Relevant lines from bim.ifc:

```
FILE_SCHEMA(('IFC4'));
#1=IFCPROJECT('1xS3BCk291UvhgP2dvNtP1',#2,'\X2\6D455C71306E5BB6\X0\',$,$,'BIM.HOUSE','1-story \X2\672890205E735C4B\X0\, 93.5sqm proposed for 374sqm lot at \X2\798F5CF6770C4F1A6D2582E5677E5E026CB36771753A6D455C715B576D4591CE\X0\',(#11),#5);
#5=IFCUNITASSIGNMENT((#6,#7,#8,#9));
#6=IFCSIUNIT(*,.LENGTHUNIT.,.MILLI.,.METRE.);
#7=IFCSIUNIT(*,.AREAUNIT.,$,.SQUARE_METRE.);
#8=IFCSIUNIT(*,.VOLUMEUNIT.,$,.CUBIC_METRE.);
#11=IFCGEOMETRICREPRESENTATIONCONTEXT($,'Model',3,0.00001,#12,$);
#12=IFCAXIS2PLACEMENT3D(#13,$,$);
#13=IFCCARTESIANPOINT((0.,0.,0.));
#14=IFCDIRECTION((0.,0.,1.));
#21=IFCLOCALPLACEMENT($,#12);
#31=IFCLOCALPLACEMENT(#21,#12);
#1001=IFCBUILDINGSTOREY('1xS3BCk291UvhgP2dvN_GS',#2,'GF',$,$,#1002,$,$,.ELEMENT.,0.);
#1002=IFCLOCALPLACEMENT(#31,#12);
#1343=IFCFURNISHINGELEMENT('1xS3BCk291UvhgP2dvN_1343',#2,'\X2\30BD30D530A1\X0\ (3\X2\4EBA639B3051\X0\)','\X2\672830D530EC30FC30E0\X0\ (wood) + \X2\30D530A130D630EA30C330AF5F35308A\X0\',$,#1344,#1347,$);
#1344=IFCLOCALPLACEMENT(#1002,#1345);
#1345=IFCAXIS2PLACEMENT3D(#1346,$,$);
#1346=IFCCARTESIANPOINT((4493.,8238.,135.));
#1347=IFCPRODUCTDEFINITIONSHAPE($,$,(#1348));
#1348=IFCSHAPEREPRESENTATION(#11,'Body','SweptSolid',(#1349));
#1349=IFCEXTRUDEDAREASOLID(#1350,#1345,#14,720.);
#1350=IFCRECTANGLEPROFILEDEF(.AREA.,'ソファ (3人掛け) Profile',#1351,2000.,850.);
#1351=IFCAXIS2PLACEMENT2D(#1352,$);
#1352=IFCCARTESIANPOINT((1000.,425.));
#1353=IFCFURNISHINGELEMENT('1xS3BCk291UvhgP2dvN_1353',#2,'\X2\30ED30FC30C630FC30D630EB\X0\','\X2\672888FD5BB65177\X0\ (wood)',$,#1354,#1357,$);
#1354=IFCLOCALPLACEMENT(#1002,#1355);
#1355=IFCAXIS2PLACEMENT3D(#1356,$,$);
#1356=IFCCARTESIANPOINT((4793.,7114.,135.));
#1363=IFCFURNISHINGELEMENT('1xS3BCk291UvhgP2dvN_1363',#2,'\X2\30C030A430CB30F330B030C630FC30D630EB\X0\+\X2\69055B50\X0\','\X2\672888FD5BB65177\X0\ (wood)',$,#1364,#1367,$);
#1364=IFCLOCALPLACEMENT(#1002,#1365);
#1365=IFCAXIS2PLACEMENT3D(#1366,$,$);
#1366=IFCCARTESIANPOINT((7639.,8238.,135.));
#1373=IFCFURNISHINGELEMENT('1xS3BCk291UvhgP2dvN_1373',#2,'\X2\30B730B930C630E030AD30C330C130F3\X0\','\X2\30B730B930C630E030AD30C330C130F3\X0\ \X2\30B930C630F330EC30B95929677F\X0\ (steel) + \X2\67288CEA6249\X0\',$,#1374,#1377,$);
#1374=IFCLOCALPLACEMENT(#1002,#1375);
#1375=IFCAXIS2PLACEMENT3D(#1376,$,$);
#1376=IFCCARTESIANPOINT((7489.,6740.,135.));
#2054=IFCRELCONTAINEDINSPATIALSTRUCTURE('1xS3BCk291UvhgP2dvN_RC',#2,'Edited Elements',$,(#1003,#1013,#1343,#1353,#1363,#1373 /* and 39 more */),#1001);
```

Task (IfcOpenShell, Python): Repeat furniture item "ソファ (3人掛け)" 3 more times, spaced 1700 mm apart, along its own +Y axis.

```python
import ifcopenshell
import ifcopenshell.api.geometry
import ifcopenshell.api.root
import ifcopenshell.util.element
import ifcopenshell.util.placement

model = ifcopenshell.open("bim.ifc")


def reuse_history(source, copy):
    """copy_class also copies each property set's owner history, people and application; keep the originals."""
    for rel in copy.IsDefinedBy:
        if rel.is_a("IfcRelDefinesByProperties") and (history := rel.RelatingPropertyDefinition.OwnerHistory):
            rel.RelatingPropertyDefinition.OwnerHistory = source.OwnerHistory
            ifcopenshell.util.element.remove_deep2(model, history)


source = model.by_guid("1xS3BCk291UvhgP2dvN_1343")
base = ifcopenshell.util.placement.get_local_placement(source.ObjectPlacement)
step = base[:3, 1] * 1700.0

for i in range(1, 4):
    copy = ifcopenshell.api.root.copy_class(model, product=source)
    copy.Representation = ifcopenshell.util.element.copy_deep(
        model, source.Representation, exclude=["IfcGeometricRepresentationContext", "IfcRepresentationMap"]
    )
    reuse_history(source, copy)
    matrix = base.copy()
    matrix[:3, 3] += i * step
    print("added at", matrix[:3, 3].round(3) + 0.0)
    ifcopenshell.api.geometry.edit_object_placement(model, product=copy, matrix=matrix, is_si=False)

model.write("bim_v2.ifc")
```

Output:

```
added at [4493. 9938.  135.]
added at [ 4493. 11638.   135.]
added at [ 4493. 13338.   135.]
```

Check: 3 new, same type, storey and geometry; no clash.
